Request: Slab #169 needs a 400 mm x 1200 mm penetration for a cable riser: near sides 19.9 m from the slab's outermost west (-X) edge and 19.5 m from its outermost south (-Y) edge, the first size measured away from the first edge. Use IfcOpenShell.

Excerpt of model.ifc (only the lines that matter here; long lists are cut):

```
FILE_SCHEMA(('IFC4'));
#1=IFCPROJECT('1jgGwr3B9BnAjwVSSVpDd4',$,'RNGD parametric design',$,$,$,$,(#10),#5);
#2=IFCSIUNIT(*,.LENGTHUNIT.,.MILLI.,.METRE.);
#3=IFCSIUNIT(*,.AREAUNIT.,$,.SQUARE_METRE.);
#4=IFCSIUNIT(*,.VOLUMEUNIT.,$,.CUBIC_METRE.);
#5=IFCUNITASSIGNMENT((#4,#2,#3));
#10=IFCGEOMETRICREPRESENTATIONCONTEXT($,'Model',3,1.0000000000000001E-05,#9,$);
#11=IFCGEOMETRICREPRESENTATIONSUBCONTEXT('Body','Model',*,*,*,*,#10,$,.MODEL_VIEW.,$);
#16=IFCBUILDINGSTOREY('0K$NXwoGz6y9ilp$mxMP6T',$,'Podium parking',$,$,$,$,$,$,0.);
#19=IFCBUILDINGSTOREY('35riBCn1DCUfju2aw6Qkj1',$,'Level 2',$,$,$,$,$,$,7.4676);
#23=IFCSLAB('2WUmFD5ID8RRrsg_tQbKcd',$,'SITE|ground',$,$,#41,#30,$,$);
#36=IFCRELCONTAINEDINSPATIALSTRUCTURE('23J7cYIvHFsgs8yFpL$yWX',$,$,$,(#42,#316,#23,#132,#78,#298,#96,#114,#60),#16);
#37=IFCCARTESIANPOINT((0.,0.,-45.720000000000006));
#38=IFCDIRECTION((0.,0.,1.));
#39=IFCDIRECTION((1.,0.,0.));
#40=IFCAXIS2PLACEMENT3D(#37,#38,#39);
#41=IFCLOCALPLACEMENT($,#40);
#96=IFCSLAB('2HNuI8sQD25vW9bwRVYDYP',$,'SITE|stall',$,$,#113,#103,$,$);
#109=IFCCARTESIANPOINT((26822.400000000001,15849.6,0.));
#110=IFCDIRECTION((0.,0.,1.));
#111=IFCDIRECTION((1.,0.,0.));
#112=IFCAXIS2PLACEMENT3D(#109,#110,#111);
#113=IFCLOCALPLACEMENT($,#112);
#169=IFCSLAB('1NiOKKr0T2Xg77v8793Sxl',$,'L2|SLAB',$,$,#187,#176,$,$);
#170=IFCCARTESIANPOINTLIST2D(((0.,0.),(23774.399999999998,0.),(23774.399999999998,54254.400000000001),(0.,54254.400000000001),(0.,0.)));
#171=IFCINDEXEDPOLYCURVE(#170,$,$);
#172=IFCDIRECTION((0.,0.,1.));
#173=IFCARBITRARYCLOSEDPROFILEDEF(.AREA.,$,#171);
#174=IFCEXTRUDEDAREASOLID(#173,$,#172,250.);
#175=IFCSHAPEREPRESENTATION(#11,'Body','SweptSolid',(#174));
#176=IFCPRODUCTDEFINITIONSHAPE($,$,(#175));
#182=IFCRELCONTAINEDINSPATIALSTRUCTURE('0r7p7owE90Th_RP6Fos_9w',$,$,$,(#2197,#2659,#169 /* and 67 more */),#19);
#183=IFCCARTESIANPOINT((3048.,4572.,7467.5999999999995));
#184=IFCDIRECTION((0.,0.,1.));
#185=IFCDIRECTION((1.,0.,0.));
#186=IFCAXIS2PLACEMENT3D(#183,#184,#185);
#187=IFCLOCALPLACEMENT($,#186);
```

```python
import numpy as np
import ifcopenshell
import ifcopenshell.api.feature
import ifcopenshell.api.geometry
import ifcopenshell.api.root
import ifcopenshell.geom
import ifcopenshell.util.placement
import ifcopenshell.util.representation
import ifcopenshell.util.shape
import ifcopenshell.util.unit

model = ifcopenshell.open("model.ifc")
unit_scale = ifcopenshell.util.unit.calculate_unit_scale(model)
settings = ifcopenshell.geom.settings()


def volume(element):
    """Net volume in cubic metres, openings subtracted."""
    shape = ifcopenshell.geom.create_shape(settings, element)
    return ifcopenshell.util.shape.get_volume(shape.geometry)


slab = model.by_guid("1NiOKKr0T2Xg77v8793Sxl")
before = volume(slab)

# Extent in the slab's own axes, in metres. The edges named are its -X and -Y sides.
slab_shape = ifcopenshell.geom.create_shape(settings, slab)
vertices = ifcopenshell.util.shape.get_vertices(slab_shape.geometry)
x_min, y_min, bottom = vertices.min(axis=0)
top = vertices[:, 2].max()

opening = ifcopenshell.api.root.create_entity(model, ifc_class="IfcOpeningElement", name="Cable riser opening", predefined_type="OPENING")
context = ifcopenshell.util.representation.get_context(model, "Model", "Body", "MODEL_VIEW")
width, depth = 0.4, 1.2
outline = [(0.0, 0.0), (width, 0.0), (width, depth), (0.0, depth), (0.0, 0.0)]
# Overshoot both faces by 50 mm so the cut is clean.
shape = ifcopenshell.api.geometry.add_slab_representation(
    model, context=context, depth=top - bottom + 0.1, polyline=outline
)
ifcopenshell.api.geometry.assign_representation(model, product=opening, representation=shape)

matrix = ifcopenshell.util.placement.get_local_placement(slab.ObjectPlacement)
matrix[:, 3] = matrix @ np.append(np.array([x_min + 19.9, y_min + 19.5, bottom - 0.05]) / unit_scale, 1.0)
ifcopenshell.api.geometry.edit_object_placement(model, product=opening, matrix=matrix, is_si=False)
ifcopenshell.api.feature.add_feature(model, feature=opening, element=slab)

after = volume(slab)

print(f"slab volume {before:.3f} -> {after:.3f} m3")

model.write("model_updated.ifc")
```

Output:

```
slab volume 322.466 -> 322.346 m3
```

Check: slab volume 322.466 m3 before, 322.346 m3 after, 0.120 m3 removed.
